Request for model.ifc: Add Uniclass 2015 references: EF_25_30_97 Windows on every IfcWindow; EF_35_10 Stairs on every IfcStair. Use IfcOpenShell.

First a look at what the model holds.

```python
import ifcopenshell

model = ifcopenshell.open("model.ifc")
print(model.schema)
print("classifications:", [c.Name for c in model.by_type("IfcClassification")])
for ifc_class in ("IfcDoor", "IfcRoof", "IfcStair", "IfcWall", "IfcWindow"):
    print(ifc_class, len(model.by_type(ifc_class)))
```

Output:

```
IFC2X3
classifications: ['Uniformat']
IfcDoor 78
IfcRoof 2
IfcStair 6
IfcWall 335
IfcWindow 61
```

```python
import ifcopenshell
import ifcopenshell.api.classification

model = ifcopenshell.open("model.ifc")

# IFC2X3 requires Source and Edition and has no link from the project to the system.
system = model.create_entity("IfcClassification", Source="NBS", Edition="2015", Name="Uniclass 2015")

codes = {
    "IfcWindow": ("EF_25_30_97", "Windows"),
    "IfcStair": ("EF_35_10", "Stairs"),
}
for ifc_class, (code, name) in codes.items():
    products = model.by_type(ifc_class)
    ifcopenshell.api.classification.add_reference(
        model, products=products, classification=system, identification=code, name=name
    )
    print(code, len(products))

model.write("model_edited.ifc")
```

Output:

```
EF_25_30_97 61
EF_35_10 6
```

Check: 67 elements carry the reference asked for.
